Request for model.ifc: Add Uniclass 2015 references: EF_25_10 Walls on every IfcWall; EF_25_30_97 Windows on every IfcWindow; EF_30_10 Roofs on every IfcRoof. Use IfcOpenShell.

First a look at what the model holds.

```python
import ifcopenshell

model = ifcopenshell.open("model.ifc")
print(model.schema)
print("classifications:", [c.Name for c in model.by_type("IfcClassification")])
for ifc_class in ("IfcDoor", "IfcRoof", "IfcStair", "IfcWall", "IfcWindow"):
    print(ifc_class, len(model.by_type(ifc_class)))
```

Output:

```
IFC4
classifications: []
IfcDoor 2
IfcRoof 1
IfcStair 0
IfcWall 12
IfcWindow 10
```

```python
import ifcopenshell
import ifcopenshell.api.classification

model = ifcopenshell.open("model.ifc")

system = ifcopenshell.api.classification.add_classification(model, classification="Uniclass 2015")

codes = {
    "IfcWall": ("EF_25_10", "Walls"),
    "IfcWindow": ("EF_25_30_97", "Windows"),
    "IfcRoof": ("EF_30_10", "Roofs"),
}
for ifc_class, (code, name) in codes.items():
    products = model.by_type(ifc_class)
    ifcopenshell.api.classification.add_reference(
        model, products=products, classification=system, identification=code, name=name
    )
    print(code, len(products))

model.write("model_updated.ifc")
```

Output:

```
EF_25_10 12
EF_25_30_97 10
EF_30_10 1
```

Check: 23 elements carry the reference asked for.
